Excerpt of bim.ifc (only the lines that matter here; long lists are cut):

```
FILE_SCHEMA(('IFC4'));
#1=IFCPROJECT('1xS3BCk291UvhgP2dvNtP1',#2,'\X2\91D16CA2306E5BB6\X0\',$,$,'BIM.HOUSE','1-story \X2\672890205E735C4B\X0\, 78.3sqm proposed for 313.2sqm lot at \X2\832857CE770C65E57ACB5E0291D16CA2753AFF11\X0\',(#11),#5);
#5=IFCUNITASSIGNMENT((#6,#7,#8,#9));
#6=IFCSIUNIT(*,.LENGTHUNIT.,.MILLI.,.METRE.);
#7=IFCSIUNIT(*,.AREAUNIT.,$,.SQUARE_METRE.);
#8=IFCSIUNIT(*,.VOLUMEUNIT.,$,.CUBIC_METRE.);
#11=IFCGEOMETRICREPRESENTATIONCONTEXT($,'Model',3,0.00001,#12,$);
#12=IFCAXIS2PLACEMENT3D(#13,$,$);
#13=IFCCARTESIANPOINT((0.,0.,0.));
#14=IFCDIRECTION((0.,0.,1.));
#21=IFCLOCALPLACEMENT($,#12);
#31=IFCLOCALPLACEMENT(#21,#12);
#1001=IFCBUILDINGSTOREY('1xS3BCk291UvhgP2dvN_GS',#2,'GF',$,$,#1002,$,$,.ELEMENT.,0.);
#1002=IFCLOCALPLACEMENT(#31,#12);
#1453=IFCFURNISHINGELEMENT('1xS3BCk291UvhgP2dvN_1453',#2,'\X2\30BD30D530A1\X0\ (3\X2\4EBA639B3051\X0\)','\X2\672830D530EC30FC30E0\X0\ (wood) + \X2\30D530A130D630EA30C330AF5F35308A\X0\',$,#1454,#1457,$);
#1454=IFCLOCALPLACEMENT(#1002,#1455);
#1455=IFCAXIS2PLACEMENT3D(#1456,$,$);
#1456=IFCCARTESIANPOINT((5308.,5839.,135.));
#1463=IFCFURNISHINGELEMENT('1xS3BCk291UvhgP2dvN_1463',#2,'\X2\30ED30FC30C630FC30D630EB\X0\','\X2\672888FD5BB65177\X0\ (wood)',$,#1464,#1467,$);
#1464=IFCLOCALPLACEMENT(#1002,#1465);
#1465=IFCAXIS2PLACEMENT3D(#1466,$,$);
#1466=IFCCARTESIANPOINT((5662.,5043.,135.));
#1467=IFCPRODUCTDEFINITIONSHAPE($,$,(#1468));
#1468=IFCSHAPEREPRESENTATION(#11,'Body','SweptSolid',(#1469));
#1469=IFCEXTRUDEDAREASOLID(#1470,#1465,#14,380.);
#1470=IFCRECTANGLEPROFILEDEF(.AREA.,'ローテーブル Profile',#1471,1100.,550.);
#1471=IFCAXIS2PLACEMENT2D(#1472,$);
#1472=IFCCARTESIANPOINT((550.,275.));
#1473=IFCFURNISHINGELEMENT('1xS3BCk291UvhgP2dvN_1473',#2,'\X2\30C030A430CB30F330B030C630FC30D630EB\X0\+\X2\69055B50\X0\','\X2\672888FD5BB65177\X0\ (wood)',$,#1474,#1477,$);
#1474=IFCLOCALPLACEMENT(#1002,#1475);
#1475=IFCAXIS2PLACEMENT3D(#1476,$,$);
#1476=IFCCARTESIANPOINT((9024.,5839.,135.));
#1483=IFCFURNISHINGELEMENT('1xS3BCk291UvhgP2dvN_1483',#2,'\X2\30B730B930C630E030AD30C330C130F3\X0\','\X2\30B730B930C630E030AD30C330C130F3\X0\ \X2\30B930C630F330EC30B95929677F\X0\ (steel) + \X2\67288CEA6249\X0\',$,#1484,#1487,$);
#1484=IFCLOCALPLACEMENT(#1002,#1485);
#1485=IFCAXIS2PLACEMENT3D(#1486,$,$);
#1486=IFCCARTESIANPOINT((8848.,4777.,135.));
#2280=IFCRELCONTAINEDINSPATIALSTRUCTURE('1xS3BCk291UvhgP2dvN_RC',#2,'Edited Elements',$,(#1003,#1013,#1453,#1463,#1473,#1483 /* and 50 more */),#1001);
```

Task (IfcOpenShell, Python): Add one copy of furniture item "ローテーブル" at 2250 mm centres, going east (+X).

```python
import numpy as np
import ifcopenshell
import ifcopenshell.api.geometry
import ifcopenshell.api.root
import ifcopenshell.util.element
import ifcopenshell.util.placement
import ifcopenshell.util.unit

model = ifcopenshell.open("bim.ifc")
unit_scale = ifcopenshell.util.unit.calculate_unit_scale(model)


def reuse_history(source, copy):
    """copy_class also copies each property set's owner history, people and application; keep the originals."""
    for rel in copy.IsDefinedBy:
        if rel.is_a("IfcRelDefinesByProperties") and (history := rel.RelatingPropertyDefinition.OwnerHistory):
            rel.RelatingPropertyDefinition.OwnerHistory = source.OwnerHistory
            ifcopenshell.util.element.remove_deep2(model, history)


source = model.by_guid("1xS3BCk291UvhgP2dvN_1463")
base = ifcopenshell.util.placement.get_local_placement(source.ObjectPlacement)
step = np.array([1.0, 0.0, 0.0]) * 2.25 / unit_scale

for i in range(1, 2):
    copy = ifcopenshell.api.root.copy_class(model, product=source)
    copy.Representation = ifcopenshell.util.element.copy_deep(
        model, source.Representation, exclude=["IfcGeometricRepresentationContext", "IfcRepresentationMap"]
    )
    reuse_history(source, copy)
    matrix = base.copy()
    matrix[:3, 3] += i * step
    print("added at", matrix[:3, 3].round(3) + 0.0)
    ifcopenshell.api.geometry.edit_object_placement(model, product=copy, matrix=matrix, is_si=False)

model.write("bim_v2.ifc")
```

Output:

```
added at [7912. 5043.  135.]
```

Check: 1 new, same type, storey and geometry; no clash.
